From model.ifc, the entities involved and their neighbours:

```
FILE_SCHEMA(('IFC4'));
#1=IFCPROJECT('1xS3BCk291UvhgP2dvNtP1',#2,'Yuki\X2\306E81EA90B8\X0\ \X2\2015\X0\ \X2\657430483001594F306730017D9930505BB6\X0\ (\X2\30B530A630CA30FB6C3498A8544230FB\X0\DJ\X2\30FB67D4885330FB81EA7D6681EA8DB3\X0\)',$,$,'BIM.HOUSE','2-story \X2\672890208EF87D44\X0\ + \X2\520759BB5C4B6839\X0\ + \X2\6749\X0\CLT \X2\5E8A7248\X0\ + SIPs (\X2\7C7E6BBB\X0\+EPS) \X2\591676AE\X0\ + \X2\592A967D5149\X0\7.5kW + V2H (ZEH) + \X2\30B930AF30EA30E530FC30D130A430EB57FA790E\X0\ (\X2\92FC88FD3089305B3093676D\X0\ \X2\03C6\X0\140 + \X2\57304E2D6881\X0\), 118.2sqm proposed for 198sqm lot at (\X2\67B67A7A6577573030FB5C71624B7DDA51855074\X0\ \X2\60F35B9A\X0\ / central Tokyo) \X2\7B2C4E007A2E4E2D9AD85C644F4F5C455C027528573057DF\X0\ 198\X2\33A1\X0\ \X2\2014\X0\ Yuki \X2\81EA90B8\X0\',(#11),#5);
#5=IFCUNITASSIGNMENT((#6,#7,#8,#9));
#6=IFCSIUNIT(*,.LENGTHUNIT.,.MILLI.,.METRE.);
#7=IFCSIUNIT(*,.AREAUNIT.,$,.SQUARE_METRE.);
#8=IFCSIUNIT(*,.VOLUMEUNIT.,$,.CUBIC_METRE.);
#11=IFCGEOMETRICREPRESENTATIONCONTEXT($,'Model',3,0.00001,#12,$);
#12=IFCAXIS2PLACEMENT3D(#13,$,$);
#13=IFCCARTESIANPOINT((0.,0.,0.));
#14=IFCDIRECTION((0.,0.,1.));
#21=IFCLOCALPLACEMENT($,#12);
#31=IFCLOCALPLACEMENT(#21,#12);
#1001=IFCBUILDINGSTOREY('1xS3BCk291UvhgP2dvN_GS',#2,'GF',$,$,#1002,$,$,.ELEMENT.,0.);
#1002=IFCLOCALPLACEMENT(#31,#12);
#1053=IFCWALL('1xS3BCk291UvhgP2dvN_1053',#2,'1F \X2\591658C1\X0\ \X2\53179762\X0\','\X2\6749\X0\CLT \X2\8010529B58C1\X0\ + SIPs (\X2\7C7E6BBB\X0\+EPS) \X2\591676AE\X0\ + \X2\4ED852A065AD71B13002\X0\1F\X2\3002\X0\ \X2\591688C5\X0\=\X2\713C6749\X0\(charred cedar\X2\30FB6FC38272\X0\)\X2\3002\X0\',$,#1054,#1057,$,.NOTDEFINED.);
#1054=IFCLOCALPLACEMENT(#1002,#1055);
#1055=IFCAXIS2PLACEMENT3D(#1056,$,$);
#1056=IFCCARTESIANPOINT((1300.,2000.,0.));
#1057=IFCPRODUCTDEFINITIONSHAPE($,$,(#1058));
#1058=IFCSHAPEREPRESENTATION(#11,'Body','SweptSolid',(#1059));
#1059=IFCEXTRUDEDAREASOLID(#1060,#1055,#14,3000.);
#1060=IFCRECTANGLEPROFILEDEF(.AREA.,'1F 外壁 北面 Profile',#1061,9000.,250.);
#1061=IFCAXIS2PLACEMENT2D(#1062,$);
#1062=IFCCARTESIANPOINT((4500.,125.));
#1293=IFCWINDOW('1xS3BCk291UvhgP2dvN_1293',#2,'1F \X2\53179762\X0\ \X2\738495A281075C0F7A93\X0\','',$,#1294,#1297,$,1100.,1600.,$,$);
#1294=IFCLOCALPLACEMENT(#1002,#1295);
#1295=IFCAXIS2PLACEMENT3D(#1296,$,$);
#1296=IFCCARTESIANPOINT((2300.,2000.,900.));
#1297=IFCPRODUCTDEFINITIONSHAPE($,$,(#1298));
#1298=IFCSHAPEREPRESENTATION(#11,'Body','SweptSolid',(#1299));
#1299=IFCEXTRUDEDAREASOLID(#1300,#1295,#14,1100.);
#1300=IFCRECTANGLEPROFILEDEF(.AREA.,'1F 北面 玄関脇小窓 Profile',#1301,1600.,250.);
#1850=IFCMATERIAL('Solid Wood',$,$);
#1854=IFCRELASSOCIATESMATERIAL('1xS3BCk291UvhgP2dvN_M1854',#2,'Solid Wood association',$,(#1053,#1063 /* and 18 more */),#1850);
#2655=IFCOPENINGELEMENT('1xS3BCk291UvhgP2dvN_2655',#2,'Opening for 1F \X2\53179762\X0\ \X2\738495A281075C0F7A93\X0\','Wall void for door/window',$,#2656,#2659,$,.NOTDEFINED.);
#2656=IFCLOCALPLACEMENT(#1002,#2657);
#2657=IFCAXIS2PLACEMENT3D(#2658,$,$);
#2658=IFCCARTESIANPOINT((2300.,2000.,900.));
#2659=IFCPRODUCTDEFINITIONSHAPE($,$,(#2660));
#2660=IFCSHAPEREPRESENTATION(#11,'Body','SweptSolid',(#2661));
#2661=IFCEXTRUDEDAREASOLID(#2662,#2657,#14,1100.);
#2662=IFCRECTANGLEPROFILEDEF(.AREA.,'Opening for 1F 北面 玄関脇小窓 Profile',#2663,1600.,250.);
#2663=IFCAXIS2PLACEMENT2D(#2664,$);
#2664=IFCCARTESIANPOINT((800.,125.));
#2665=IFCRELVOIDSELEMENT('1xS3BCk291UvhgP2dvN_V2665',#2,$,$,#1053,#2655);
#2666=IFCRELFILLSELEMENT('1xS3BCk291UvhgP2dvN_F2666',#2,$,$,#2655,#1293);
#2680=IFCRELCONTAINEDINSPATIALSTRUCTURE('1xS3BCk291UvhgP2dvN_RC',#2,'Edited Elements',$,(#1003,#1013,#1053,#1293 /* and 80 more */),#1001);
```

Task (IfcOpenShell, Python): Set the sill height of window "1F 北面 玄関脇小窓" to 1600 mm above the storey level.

```python
import numpy as np
import ifcopenshell
import ifcopenshell.api.geometry
import ifcopenshell.geom
import ifcopenshell.util.element
import ifcopenshell.util.placement
import ifcopenshell.util.shape
import ifcopenshell.util.unit

model = ifcopenshell.open("model.ifc")
unit_scale = ifcopenshell.util.unit.calculate_unit_scale(model)

window = model.by_guid("1xS3BCk291UvhgP2dvN_1293")
opening = window.FillsVoids[0].RelatingOpeningElement
storey = ifcopenshell.util.element.get_container(window, ifc_class="IfcBuildingStorey")
level = ifcopenshell.util.placement.get_local_placement(storey.ObjectPlacement)[2, 3]

# The opening's origin need not be at the sill, so measure its lowest point.
shape = ifcopenshell.geom.create_shape(ifcopenshell.geom.settings(), opening)
bottom = ifcopenshell.util.shape.get_shape_bottom_elevation(shape, shape.geometry) / unit_scale
dz = level + 1.6 / unit_scale - bottom

shift = np.array([0.0, 0.0, dz])
# The window is not placed relative to its opening, so move both.
for product in (opening, window):
    matrix = ifcopenshell.util.placement.get_local_placement(product.ObjectPlacement)
    matrix[:3, 3] += shift
    ifcopenshell.api.geometry.edit_object_placement(model, product=product, matrix=matrix, is_si=False)

print(f"moved by {dz * unit_scale:+.3f} m")

model.write("model_updated.ifc")
```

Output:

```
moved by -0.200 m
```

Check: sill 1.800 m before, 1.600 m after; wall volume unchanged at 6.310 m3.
